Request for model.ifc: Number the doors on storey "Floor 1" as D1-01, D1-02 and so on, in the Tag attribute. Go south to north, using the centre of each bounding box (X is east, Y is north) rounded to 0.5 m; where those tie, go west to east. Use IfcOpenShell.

First a look at what the model holds.

```python
import ifcopenshell
import ifcopenshell.util.element
import ifcopenshell.util.placement

model = ifcopenshell.open("model.ifc")
print(model.schema)
storey = next(s for s in model.by_type("IfcBuildingStorey") if s.Name == "Floor 1")
doors = [e for e in ifcopenshell.util.element.get_decomposition(storey) if e.is_a("IfcDoor")]
for e in sorted(doors, key=lambda e: e.id()):
    origin = ifcopenshell.util.placement.get_local_placement(e.ObjectPlacement)[:3, 3]
    print(e.id(), e.Tag, e.Name, origin.round(2) + 0.0, sep=" | ")
```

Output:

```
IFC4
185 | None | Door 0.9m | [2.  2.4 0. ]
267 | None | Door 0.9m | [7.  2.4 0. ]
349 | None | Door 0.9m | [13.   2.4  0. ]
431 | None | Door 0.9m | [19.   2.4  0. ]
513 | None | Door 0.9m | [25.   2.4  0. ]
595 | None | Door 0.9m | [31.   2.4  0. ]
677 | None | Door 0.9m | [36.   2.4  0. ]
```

```python
import ifcopenshell
import ifcopenshell.geom
import ifcopenshell.util.element
import ifcopenshell.util.shape

model = ifcopenshell.open("model.ifc")
settings = ifcopenshell.geom.settings()
settings.set("use-world-coords", True)


def centre(element):
    shape = ifcopenshell.geom.create_shape(settings, element)
    return ifcopenshell.util.shape.get_bbox_centroid(shape.geometry)


storey = next(s for s in model.by_type("IfcBuildingStorey") if s.Name == "Floor 1")
doors = [e for e in ifcopenshell.util.element.get_decomposition(storey) if e.is_a("IfcDoor")]

# Insertion points can sit at a corner or the storey origin, so sort by the geometry (in metres).
centres = {e: centre(e) for e in doors}
doors.sort(key=lambda e: (round(centres[e][1] / 0.5), centres[e][0]))

for i, e in enumerate(doors, start=1):
    number = f"D1-{i:02d}"
    e.Tag = number
    print(e.id(), number)

model.write("model_rev.ifc")
```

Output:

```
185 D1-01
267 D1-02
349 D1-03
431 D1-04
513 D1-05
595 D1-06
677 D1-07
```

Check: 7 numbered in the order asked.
